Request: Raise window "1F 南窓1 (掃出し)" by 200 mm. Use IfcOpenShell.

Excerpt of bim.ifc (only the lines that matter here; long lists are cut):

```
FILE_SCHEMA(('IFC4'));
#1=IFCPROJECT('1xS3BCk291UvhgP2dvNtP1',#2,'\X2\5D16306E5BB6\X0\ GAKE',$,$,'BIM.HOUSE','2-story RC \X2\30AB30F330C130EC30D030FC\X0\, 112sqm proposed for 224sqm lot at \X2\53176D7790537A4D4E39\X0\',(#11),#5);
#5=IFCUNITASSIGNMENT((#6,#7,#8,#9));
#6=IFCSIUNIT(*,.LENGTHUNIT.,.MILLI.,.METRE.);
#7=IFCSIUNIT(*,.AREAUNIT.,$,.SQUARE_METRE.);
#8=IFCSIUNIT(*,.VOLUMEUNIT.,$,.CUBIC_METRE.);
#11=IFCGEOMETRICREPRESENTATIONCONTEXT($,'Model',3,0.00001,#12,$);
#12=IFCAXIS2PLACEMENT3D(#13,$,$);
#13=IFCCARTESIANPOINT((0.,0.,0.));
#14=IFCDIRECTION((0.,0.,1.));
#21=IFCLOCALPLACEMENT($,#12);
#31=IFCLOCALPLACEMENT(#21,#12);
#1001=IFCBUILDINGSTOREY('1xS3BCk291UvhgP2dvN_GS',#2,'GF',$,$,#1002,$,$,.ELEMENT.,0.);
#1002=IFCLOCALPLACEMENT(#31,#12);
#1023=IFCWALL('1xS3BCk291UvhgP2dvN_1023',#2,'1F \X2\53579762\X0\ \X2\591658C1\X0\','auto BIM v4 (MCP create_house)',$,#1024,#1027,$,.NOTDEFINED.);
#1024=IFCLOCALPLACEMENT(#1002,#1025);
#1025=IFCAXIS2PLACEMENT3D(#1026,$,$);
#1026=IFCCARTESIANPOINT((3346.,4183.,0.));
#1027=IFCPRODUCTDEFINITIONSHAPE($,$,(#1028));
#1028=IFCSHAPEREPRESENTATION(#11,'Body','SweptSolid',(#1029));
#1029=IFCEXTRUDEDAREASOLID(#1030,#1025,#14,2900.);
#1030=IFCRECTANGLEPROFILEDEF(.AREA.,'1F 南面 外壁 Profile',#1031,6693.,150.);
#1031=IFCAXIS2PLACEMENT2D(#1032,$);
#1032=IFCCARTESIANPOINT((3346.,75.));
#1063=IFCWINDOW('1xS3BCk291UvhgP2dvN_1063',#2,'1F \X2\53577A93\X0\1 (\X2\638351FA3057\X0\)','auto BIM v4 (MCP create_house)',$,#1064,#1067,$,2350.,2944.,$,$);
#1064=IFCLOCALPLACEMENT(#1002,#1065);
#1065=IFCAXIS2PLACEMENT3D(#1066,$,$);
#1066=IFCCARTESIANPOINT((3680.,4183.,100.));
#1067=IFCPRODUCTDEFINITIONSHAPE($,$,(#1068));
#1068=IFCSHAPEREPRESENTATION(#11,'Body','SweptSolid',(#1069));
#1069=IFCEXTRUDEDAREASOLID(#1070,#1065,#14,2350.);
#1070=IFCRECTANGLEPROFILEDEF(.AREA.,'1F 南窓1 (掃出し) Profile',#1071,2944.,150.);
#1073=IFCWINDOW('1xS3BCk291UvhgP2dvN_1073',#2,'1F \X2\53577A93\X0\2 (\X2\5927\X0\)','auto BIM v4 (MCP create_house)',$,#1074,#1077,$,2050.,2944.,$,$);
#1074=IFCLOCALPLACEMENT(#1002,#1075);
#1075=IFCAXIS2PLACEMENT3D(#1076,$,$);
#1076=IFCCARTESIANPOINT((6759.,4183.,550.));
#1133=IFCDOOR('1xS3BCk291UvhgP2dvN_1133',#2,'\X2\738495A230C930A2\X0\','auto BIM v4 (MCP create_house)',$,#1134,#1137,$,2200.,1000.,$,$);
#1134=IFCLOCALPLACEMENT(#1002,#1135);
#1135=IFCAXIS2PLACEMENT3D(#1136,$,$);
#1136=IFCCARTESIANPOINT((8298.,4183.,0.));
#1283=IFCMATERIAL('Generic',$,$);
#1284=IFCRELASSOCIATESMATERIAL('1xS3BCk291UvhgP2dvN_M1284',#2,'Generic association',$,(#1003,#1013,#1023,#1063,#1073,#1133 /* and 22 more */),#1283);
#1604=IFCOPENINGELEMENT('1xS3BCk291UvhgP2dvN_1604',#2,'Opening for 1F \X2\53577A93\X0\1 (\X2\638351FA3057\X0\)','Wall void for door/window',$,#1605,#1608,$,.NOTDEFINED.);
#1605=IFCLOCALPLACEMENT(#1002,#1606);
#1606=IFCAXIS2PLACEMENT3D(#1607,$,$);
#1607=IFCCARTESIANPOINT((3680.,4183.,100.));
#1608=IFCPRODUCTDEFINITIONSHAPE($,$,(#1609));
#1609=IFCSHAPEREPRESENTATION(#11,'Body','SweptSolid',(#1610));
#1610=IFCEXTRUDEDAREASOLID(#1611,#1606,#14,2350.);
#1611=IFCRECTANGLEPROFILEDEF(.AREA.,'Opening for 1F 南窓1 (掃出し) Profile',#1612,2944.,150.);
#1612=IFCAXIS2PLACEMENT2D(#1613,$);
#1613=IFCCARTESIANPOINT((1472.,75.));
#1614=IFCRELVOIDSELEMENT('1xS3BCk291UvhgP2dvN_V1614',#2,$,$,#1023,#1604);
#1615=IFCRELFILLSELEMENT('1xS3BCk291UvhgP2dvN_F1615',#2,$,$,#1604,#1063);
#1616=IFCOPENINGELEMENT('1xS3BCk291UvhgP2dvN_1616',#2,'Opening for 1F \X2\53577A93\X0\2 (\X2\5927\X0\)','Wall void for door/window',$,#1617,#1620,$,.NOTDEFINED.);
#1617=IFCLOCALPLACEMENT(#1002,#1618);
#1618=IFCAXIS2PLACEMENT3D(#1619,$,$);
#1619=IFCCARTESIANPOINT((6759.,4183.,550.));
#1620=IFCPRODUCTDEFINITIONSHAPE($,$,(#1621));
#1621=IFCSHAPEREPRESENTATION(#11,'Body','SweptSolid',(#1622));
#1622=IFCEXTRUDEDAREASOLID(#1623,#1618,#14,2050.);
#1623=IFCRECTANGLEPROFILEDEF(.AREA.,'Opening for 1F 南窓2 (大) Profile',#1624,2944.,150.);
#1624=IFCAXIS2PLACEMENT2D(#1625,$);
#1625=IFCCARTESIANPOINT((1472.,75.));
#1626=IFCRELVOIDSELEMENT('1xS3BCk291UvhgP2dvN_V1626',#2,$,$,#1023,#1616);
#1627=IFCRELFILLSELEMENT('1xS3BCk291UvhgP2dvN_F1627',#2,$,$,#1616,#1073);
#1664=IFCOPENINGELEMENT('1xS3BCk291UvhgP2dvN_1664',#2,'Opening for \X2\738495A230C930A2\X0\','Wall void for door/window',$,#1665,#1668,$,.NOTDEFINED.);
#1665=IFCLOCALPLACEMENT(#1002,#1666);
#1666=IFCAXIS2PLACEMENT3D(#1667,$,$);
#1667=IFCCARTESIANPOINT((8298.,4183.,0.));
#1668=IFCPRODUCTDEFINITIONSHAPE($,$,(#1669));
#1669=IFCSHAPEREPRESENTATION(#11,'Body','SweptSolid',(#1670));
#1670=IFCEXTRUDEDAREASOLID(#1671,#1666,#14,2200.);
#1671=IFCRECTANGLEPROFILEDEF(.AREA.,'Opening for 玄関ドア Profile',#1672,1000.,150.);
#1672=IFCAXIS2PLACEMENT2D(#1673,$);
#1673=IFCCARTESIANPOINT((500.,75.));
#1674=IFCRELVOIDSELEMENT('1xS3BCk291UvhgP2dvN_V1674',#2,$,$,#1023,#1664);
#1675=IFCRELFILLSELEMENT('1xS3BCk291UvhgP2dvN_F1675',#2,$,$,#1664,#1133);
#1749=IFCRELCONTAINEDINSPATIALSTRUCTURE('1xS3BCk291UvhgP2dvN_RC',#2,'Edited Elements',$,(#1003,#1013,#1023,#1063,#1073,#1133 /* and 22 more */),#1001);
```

```python
import numpy as np
import ifcopenshell
import ifcopenshell.api.geometry
import ifcopenshell.util.placement
import ifcopenshell.util.unit

model = ifcopenshell.open("bim.ifc")
unit_scale = ifcopenshell.util.unit.calculate_unit_scale(model)

window = model.by_id(1063)
opening = window.FillsVoids[0].RelatingOpeningElement
dz = 200.0

shift = np.array([0.0, 0.0, dz])
# The window is not placed relative to its opening, so move both.
for product in (opening, window):
    matrix = ifcopenshell.util.placement.get_local_placement(product.ObjectPlacement)
    matrix[:3, 3] += shift
    ifcopenshell.api.geometry.edit_object_placement(model, product=product, matrix=matrix, is_si=False)

print(f"moved by {dz * unit_scale:+.3f} m")

model.write("bim_v2.ifc")
```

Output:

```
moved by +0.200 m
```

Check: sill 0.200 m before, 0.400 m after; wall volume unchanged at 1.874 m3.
